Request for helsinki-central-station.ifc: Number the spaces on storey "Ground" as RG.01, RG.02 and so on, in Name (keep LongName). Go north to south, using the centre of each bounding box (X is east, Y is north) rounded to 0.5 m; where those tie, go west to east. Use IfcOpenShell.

First a look at what the model holds.

```python
import ifcopenshell
import ifcopenshell.util.element
import ifcopenshell.util.placement

model = ifcopenshell.open("helsinki-central-station.ifc")
print(model.schema)
storey = next(s for s in model.by_type("IfcBuildingStorey") if s.Name == "Ground")
spaces = [e for e in ifcopenshell.util.element.get_decomposition(storey) if e.is_a("IfcSpace")]
for e in sorted(spaces, key=lambda e: e.id()):
    origin = ifcopenshell.util.placement.get_local_placement(e.ObjectPlacement)[:3, 3]
    print(e.id(), e.Name, e.LongName, origin.round(2) + 0.0, sep=" | ")
```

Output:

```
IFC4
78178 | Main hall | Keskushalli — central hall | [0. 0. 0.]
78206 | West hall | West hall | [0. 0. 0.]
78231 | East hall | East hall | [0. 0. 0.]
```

```python
import ifcopenshell
import ifcopenshell.geom
import ifcopenshell.util.element
import ifcopenshell.util.shape

model = ifcopenshell.open("helsinki-central-station.ifc")
settings = ifcopenshell.geom.settings()
settings.set("use-world-coords", True)


def centre(element):
    shape = ifcopenshell.geom.create_shape(settings, element)
    return ifcopenshell.util.shape.get_bbox_centroid(shape.geometry)


storey = next(s for s in model.by_type("IfcBuildingStorey") if s.Name == "Ground")
spaces = [e for e in ifcopenshell.util.element.get_decomposition(storey) if e.is_a("IfcSpace")]

# Insertion points can sit at a corner or the storey origin, so sort by the geometry (in metres).
centres = {e: centre(e) for e in spaces}
spaces.sort(key=lambda e: (-round(centres[e][1] / 0.5), centres[e][0]))

for i, e in enumerate(spaces, start=1):
    number = f"RG.{i:02d}"
    e.Name = number
    print(e.id(), number)

model.write("helsinki-central-station_updated.ifc")
```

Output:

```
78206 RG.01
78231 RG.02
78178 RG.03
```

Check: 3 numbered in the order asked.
